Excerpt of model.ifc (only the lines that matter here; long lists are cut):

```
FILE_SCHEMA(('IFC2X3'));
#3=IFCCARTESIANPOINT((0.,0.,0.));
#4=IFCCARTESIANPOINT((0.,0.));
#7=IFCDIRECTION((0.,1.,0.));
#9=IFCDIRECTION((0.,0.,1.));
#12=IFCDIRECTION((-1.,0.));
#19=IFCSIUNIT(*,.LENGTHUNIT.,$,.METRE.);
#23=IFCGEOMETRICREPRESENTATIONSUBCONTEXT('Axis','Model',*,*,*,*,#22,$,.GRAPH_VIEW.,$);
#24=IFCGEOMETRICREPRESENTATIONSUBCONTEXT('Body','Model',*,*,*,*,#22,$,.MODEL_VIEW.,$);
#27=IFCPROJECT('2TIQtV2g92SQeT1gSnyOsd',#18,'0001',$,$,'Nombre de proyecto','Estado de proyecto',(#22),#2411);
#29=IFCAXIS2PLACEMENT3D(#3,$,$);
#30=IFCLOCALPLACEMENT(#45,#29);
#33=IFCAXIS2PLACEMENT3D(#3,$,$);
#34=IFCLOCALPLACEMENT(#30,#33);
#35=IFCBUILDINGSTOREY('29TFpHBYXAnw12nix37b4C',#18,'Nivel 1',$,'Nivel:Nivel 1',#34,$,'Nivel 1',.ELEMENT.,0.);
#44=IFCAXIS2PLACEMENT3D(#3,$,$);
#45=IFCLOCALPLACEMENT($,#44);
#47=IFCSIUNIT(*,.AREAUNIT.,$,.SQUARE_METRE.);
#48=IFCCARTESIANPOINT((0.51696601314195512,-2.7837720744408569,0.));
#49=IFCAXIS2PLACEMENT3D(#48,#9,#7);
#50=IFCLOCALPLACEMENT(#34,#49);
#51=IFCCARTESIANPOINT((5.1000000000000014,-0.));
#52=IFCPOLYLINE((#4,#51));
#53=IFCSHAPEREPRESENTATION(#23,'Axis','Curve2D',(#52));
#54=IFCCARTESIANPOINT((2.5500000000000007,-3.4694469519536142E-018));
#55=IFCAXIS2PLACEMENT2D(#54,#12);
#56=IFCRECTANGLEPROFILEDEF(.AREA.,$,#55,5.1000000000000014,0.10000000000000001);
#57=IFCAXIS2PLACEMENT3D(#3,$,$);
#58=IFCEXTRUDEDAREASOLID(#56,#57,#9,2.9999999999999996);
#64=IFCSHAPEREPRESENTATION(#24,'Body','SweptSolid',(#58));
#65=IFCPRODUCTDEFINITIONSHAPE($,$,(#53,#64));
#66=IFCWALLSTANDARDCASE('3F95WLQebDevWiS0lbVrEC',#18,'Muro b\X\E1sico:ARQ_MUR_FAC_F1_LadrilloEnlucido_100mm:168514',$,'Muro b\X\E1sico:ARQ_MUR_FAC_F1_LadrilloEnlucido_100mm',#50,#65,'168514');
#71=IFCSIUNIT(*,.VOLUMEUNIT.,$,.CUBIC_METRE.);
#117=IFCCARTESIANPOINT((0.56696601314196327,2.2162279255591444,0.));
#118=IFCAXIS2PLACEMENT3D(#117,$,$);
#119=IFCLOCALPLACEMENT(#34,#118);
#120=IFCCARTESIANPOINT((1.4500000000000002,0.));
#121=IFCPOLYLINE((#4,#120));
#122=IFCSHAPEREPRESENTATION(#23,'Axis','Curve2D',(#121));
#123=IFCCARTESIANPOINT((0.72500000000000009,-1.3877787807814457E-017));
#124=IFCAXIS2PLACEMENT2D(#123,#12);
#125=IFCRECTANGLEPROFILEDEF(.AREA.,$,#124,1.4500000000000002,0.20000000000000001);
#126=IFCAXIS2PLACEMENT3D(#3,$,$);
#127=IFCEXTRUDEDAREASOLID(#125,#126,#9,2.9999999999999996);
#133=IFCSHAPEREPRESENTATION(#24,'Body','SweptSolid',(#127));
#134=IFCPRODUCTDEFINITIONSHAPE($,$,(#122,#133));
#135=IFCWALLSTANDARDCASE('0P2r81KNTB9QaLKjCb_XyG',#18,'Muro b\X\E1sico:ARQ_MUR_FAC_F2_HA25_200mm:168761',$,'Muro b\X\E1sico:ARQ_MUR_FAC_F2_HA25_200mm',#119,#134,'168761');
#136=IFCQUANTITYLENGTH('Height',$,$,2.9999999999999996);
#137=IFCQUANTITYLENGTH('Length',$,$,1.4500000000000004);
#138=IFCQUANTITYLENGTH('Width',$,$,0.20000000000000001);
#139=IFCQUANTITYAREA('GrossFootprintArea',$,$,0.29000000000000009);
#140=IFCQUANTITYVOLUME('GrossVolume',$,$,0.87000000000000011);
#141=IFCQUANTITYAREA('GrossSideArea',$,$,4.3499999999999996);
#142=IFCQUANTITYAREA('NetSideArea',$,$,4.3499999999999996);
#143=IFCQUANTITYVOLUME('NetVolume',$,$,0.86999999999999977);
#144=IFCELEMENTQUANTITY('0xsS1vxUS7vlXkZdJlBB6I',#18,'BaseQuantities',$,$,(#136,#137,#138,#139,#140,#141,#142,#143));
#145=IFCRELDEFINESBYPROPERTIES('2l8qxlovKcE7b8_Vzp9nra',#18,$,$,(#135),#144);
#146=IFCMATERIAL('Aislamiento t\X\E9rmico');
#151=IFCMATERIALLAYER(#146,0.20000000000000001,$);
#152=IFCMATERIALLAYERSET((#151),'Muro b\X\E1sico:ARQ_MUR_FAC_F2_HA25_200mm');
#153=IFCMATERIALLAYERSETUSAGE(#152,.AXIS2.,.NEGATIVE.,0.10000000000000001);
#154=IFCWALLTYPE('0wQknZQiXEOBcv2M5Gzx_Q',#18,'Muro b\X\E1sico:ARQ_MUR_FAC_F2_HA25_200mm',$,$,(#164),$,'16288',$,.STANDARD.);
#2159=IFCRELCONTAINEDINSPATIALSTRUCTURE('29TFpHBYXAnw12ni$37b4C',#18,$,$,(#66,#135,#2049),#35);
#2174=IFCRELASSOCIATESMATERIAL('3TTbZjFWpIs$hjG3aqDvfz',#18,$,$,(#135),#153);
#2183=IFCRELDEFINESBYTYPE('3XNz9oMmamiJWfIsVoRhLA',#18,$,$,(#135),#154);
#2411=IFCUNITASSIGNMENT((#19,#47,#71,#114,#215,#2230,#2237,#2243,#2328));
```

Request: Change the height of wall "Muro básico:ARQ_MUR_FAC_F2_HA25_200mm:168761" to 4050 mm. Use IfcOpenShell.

```python
import ifcopenshell
import ifcopenshell.api.pset
import ifcopenshell.geom
import ifcopenshell.util.element
import ifcopenshell.util.representation
import ifcopenshell.util.shape
import ifcopenshell.util.unit

model = ifcopenshell.open("model.ifc")
unit_scale = ifcopenshell.util.unit.calculate_unit_scale(model)
area_scale = ifcopenshell.util.unit.calculate_unit_scale(model, "AREAUNIT")
volume_scale = ifcopenshell.util.unit.calculate_unit_scale(model, "VOLUMEUNIT")
settings = ifcopenshell.geom.settings()


def volume(element):
    """Net volume in cubic metres, openings subtracted."""
    shape = ifcopenshell.geom.create_shape(settings, element)
    return ifcopenshell.util.shape.get_volume(shape.geometry)


wall = model.by_guid("0P2r81KNTB9QaLKjCb_XyG")
before = volume(wall)

body = ifcopenshell.util.representation.get_representation(wall, "Model", "Body")
solid = body.Items[0]
old_height = solid.Depth
solid.Depth = 4.05 / unit_scale
after = volume(wall)
thickness = 0.2  # wall thickness in metres

# Update the stored height, areas and volumes.
qto = model.by_id(ifcopenshell.util.element.get_pset(wall, "BaseQuantities", should_inherit=False)["id"])
ifcopenshell.api.pset.edit_qto(model, qto=qto, properties={
    "Height": solid.Depth,
    "GrossVolume": ifcopenshell.util.element.get_pset(wall, "BaseQuantities", "GrossVolume") * solid.Depth / old_height,
    "GrossSideArea": ifcopenshell.util.element.get_pset(wall, "BaseQuantities", "GrossSideArea") * solid.Depth / old_height,
    "NetSideArea": after / thickness / area_scale,
    "NetVolume": after / volume_scale,
})

print(f"height {old_height:g} -> {solid.Depth:g}, volume {before:.3f} -> {after:.3f} m3")

model.write("model_edited.ifc")
```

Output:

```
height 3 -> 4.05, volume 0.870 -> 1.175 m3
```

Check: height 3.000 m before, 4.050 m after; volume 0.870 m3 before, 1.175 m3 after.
